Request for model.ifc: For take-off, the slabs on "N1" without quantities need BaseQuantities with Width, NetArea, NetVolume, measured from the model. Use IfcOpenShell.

First a look at what the model holds.

```python
import ifcopenshell
import ifcopenshell.util.element
import ifcopenshell.util.unit

model = ifcopenshell.open("model.ifc")
print(model.schema)
for unit_type in ("LENGTHUNIT", "AREAUNIT", "VOLUMEUNIT"):
    print(unit_type, ifcopenshell.util.unit.calculate_unit_scale(model, unit_type))
storey = next(s for s in model.by_type("IfcBuildingStorey") if s.Name == "N1")
slabs = [e for e in ifcopenshell.util.element.get_decomposition(storey) if e.is_a("IfcSlab")]
for e in sorted(slabs, key=lambda e: e.id()):
    print(e.id(), e.is_a(), e.Name, list(ifcopenshell.util.element.get_psets(e, qtos_only=True)), sep=" | ")
```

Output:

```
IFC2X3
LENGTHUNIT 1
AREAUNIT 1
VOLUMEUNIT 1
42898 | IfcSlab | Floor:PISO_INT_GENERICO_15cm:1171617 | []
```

```python
import ifcopenshell
import ifcopenshell.api.pset
import ifcopenshell.geom
import ifcopenshell.util.element
import ifcopenshell.util.shape
import ifcopenshell.util.unit

model = ifcopenshell.open("model.ifc")
unit_scale = ifcopenshell.util.unit.calculate_unit_scale(model)
area_scale = ifcopenshell.util.unit.calculate_unit_scale(model, "AREAUNIT")
volume_scale = ifcopenshell.util.unit.calculate_unit_scale(model, "VOLUMEUNIT")
settings = ifcopenshell.geom.settings()

storey = next(s for s in model.by_type("IfcBuildingStorey") if s.Name == "N1")
slabs = [e for e in ifcopenshell.util.element.get_decomposition(storey) if e.is_a("IfcSlab")]

for e in sorted(slabs, key=lambda e: e.id()):
    if ifcopenshell.util.element.get_psets(e, qtos_only=True, should_inherit=False):
        continue
    # Geometry comes back in metres, in the element's own axes.
    shape = ifcopenshell.geom.create_shape(settings, e)
    values = {
        "Width": ifcopenshell.util.shape.get_z(shape.geometry) / unit_scale,
        "NetArea": ifcopenshell.util.shape.get_footprint_area(shape.geometry) / area_scale,
        "NetVolume": ifcopenshell.util.shape.get_volume(shape.geometry) / volume_scale,
    }
    qto = ifcopenshell.api.pset.add_qto(model, product=e, name="BaseQuantities")
    ifcopenshell.api.pset.edit_qto(model, qto=qto, properties=values)
    print(e.id(), {k: round(v, 3) for k, v in values.items()})

model.write("model-out.ifc")
```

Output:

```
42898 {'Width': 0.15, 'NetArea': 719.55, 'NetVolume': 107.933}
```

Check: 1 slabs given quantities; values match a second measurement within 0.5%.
